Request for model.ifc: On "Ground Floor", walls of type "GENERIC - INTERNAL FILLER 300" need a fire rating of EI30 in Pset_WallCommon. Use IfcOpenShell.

First a look at what the model holds.

```python
import ifcopenshell
import ifcopenshell.util.element

model = ifcopenshell.open("model.ifc")
print(model.schema)
storey = next(s for s in model.by_type("IfcBuildingStorey") if s.Name == "Ground Floor")
walls = [e for e in ifcopenshell.util.element.get_decomposition(storey) if e.is_a("IfcWall")]
seen = {}
for e in walls:
    element_type = ifcopenshell.util.element.get_type(e)
    key = (element_type.Name if element_type != e and element_type else None, ifcopenshell.util.element.get_pset(e, "Pset_WallCommon", "FireRating"))
    seen[key] = seen.get(key, 0) + 1
for (name, value), count in sorted(seen.items(), key=str):
    print(count, "x", name, "|", value)
```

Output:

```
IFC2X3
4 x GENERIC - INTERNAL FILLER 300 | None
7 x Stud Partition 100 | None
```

```python
import ifcopenshell
import ifcopenshell.api.pset
import ifcopenshell.util.element

model = ifcopenshell.open("model.ifc")

storey = next(s for s in model.by_type("IfcBuildingStorey") if s.Name == "Ground Floor")
walls = [e for e in ifcopenshell.util.element.get_decomposition(storey) if e.is_a("IfcWall")]

count = 0
for e in walls:
    element_type = ifcopenshell.util.element.get_type(e)
    if element_type in (None, e) or element_type.Name != "GENERIC - INTERNAL FILLER 300":
        continue
    # add_pset returns the element's existing set when there is one.
    pset = ifcopenshell.api.pset.add_pset(model, product=e, name="Pset_WallCommon")
    ifcopenshell.api.pset.edit_pset(model, pset=pset, properties={"FireRating": "EI30"})
    count += 1

print(count, "walls updated")

model.write("model_edited.ifc")
```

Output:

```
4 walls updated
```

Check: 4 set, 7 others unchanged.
